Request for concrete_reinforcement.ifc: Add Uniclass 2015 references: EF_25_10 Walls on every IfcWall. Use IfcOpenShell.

First a look at what the model holds.

```python
import ifcopenshell

model = ifcopenshell.open("concrete_reinforcement.ifc")
print(model.schema)
print("classifications:", [c.Name for c in model.by_type("IfcClassification")])
for ifc_class in ("IfcDoor", "IfcRoof", "IfcStair", "IfcWall", "IfcWindow"):
    print(ifc_class, len(model.by_type(ifc_class)))
```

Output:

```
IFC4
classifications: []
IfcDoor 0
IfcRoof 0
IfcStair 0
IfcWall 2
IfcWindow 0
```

```python
import ifcopenshell
import ifcopenshell.api.classification

model = ifcopenshell.open("concrete_reinforcement.ifc")

system = ifcopenshell.api.classification.add_classification(model, classification="Uniclass 2015")

codes = {
    "IfcWall": ("EF_25_10", "Walls"),
}
for ifc_class, (code, name) in codes.items():
    products = model.by_type(ifc_class)
    ifcopenshell.api.classification.add_reference(
        model, products=products, classification=system, identification=code, name=name
    )
    print(code, len(products))

model.write("concrete_reinforcement_rev.ifc")
```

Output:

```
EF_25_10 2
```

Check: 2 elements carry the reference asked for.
